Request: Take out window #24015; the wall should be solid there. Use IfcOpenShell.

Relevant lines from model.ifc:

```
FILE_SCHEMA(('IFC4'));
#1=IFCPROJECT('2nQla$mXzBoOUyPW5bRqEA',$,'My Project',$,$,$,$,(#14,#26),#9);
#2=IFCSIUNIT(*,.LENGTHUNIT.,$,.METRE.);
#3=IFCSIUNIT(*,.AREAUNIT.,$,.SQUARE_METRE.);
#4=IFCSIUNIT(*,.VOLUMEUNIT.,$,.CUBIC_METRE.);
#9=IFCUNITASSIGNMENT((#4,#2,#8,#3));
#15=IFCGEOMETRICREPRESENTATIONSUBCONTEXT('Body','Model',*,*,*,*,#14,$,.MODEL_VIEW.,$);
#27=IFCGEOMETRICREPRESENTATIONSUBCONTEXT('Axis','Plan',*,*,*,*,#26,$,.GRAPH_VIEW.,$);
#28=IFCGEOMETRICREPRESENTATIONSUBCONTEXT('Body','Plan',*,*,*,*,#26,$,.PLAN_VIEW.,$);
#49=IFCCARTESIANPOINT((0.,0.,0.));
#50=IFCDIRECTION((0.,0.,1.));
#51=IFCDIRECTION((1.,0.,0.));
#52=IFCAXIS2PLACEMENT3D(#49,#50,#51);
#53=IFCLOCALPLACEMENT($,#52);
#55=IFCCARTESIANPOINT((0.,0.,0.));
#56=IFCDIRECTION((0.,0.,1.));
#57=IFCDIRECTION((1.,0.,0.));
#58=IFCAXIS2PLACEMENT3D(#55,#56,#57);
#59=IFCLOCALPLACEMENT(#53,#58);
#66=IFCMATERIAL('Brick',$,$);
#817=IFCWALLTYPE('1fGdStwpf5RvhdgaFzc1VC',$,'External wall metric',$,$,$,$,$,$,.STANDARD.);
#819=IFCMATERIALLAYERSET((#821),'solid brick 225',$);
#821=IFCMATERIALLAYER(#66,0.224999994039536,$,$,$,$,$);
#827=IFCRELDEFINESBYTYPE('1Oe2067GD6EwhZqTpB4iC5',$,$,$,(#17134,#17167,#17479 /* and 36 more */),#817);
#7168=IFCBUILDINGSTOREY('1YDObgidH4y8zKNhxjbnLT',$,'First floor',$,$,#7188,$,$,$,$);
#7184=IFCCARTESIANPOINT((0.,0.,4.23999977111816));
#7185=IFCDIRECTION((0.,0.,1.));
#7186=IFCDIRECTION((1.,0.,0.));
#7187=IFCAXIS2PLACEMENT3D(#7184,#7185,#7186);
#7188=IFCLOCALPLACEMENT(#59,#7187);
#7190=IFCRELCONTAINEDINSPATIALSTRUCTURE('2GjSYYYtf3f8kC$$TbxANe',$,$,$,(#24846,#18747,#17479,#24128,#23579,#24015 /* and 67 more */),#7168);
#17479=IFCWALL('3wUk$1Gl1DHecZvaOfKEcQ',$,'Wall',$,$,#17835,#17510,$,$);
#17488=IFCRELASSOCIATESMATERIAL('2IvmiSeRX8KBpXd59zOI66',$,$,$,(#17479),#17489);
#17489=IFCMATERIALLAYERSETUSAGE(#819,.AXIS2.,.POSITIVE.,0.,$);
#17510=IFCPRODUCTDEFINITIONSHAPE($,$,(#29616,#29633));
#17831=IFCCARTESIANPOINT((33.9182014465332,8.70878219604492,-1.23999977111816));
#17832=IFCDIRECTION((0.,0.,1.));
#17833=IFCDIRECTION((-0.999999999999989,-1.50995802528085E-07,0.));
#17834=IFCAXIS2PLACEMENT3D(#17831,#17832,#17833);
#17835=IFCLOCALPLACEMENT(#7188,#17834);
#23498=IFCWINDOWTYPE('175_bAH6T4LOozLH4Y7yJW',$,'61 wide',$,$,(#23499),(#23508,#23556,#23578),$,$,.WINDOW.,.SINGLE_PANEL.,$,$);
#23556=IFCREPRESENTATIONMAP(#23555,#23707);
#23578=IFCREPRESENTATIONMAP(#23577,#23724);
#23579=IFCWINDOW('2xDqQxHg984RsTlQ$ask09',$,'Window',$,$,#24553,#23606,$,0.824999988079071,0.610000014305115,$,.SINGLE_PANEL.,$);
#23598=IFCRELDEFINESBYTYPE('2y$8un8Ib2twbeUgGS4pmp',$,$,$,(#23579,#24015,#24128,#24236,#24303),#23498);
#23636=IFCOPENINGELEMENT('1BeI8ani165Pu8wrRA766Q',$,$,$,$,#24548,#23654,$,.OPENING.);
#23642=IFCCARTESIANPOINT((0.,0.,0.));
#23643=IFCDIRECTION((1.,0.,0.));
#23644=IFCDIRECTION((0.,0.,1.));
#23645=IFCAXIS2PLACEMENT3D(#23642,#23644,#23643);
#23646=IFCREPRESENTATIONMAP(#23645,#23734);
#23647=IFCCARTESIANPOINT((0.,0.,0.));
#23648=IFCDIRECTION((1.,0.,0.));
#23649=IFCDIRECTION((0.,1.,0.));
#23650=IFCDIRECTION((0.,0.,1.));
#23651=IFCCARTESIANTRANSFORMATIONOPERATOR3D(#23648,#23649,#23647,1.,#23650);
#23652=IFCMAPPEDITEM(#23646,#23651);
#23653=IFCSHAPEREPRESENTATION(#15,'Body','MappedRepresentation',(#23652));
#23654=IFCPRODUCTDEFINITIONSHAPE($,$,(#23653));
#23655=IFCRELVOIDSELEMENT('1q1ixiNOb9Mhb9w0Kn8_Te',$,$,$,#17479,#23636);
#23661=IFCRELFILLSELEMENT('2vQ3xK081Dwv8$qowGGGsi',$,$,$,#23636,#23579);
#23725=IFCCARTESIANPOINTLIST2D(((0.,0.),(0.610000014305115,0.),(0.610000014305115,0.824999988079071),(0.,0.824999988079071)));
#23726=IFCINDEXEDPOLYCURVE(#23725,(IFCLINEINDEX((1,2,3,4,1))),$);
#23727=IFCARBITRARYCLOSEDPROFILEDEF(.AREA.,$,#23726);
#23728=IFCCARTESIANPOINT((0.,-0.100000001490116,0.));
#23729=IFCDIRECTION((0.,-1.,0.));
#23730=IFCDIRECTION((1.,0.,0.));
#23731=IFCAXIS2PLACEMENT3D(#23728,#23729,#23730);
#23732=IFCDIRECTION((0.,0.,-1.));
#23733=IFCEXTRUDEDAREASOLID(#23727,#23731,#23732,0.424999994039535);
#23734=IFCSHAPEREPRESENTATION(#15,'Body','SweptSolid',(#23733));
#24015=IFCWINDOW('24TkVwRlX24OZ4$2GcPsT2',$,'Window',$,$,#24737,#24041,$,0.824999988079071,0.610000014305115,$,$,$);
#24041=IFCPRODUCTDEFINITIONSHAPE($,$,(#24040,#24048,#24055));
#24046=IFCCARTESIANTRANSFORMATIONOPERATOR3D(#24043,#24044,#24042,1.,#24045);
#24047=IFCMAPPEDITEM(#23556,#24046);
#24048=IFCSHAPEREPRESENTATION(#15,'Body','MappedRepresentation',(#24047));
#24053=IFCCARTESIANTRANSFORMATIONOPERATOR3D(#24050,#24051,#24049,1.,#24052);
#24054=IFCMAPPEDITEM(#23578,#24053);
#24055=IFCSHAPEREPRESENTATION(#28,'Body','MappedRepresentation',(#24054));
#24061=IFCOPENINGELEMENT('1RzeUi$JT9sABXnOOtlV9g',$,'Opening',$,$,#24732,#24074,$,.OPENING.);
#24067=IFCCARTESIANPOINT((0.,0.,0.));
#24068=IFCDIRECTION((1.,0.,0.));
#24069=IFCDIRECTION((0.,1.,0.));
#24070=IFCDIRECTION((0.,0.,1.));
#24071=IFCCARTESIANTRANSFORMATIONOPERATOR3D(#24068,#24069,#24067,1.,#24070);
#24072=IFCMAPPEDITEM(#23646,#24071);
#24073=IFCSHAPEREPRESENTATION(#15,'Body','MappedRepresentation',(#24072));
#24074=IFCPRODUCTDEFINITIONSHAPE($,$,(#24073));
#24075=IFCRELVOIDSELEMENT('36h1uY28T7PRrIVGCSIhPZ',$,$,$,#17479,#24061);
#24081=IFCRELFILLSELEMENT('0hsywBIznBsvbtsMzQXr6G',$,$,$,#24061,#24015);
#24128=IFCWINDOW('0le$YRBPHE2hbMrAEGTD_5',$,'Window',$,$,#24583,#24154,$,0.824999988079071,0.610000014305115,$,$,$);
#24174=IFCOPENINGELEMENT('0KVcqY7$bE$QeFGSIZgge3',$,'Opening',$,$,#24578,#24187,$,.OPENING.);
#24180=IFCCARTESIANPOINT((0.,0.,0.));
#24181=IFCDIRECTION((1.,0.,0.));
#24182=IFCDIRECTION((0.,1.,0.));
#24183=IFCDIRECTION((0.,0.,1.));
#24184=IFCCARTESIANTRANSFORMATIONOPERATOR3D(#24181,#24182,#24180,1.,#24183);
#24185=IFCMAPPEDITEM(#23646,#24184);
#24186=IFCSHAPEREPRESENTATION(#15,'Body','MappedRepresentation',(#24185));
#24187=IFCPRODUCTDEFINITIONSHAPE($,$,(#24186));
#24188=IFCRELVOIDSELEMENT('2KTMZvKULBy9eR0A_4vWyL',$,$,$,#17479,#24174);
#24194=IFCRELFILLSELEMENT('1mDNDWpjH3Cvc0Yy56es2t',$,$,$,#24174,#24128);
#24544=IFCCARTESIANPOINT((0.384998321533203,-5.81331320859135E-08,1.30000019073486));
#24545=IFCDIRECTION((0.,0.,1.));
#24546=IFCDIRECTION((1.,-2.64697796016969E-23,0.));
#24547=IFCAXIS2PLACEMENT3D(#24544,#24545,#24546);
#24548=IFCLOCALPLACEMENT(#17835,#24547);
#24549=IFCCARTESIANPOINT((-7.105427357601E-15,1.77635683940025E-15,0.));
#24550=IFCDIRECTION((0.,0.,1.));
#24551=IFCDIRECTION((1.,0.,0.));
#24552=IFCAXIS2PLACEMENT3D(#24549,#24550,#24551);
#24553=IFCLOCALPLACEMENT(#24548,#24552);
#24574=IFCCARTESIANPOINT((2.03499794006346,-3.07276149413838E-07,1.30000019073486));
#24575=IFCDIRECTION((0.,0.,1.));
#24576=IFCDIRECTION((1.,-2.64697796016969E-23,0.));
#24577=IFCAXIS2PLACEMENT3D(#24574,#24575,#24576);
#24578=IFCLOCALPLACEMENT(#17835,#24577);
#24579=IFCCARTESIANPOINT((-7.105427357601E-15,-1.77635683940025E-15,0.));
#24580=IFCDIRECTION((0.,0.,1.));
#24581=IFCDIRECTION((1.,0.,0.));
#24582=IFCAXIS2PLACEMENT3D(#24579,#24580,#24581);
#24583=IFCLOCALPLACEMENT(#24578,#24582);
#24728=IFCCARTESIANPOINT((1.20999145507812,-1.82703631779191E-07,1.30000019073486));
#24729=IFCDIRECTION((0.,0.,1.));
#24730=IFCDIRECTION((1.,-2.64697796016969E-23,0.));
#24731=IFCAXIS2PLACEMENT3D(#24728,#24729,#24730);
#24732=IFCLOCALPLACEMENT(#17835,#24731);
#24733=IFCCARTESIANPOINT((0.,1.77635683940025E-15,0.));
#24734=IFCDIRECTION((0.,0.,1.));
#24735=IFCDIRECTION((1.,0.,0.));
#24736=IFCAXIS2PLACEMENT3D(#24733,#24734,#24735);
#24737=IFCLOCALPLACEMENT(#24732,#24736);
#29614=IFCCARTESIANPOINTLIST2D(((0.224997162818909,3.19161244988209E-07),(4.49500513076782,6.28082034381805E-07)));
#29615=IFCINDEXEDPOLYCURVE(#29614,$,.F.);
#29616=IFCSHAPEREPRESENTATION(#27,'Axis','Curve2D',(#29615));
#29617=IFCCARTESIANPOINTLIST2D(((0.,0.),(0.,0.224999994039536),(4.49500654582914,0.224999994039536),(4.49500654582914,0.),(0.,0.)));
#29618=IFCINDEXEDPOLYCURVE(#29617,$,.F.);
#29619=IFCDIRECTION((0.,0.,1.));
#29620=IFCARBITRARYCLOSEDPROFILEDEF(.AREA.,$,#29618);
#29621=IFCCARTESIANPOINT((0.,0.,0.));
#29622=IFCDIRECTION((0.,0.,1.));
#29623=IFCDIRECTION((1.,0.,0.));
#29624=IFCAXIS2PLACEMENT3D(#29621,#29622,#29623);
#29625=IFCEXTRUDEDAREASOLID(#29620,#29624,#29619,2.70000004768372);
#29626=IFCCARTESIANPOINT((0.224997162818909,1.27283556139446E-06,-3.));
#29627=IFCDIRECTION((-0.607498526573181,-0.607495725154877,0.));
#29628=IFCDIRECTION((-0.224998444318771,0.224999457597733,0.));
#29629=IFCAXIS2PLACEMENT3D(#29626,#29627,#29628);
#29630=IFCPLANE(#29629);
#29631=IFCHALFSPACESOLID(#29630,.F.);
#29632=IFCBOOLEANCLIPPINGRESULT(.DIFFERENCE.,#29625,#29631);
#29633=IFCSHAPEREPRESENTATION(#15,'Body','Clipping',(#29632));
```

```python
import ifcopenshell
import ifcopenshell.api.feature
import ifcopenshell.api.root
import ifcopenshell.geom
import ifcopenshell.util.shape

model = ifcopenshell.open("model.ifc")
settings = ifcopenshell.geom.settings()


def volume(element):
    """Net volume in cubic metres, openings subtracted."""
    shape = ifcopenshell.geom.create_shape(settings, element)
    return ifcopenshell.util.shape.get_volume(shape.geometry)


window = model.by_id(24015)
opening = window.FillsVoids[0].RelatingOpeningElement
wall = opening.VoidsElements[0].RelatingBuildingElement
before = volume(wall)

ifcopenshell.api.root.remove_product(model, product=window)
ifcopenshell.api.feature.remove_feature(model, feature=opening)

after = volume(wall)

print(f"wall volume {before:.3f} -> {after:.3f} m3")

model.write("model-out.ifc")
```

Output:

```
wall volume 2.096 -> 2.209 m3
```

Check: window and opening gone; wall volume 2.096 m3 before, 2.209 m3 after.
